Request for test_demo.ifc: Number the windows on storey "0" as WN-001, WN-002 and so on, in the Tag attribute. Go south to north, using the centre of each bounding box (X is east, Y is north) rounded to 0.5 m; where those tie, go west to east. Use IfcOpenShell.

First a look at what the model holds.

```python
import ifcopenshell
import ifcopenshell.util.element
import ifcopenshell.util.placement

model = ifcopenshell.open("test_demo.ifc")
print(model.schema)
storey = next(s for s in model.by_type("IfcBuildingStorey") if s.Name == "0")
windows = [e for e in ifcopenshell.util.element.get_decomposition(storey) if e.is_a("IfcWindow")]
for e in sorted(windows, key=lambda e: e.id()):
    origin = ifcopenshell.util.placement.get_local_placement(e.ObjectPlacement)[:3, 3]
    print(e.id(), e.Tag, e.Name, origin.round(2) + 0.0, sep=" | ")
```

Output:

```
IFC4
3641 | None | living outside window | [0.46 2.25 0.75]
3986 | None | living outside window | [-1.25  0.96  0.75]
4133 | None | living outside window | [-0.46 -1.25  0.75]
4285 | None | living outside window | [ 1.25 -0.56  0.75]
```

```python
import ifcopenshell
import ifcopenshell.geom
import ifcopenshell.util.element
import ifcopenshell.util.shape

model = ifcopenshell.open("test_demo.ifc")
settings = ifcopenshell.geom.settings()
settings.set("use-world-coords", True)


def centre(element):
    shape = ifcopenshell.geom.create_shape(settings, element)
    return ifcopenshell.util.shape.get_bbox_centroid(shape.geometry)


storey = next(s for s in model.by_type("IfcBuildingStorey") if s.Name == "0")
windows = [e for e in ifcopenshell.util.element.get_decomposition(storey) if e.is_a("IfcWindow")]

# Insertion points can sit at a corner or the storey origin, so sort by the geometry (in metres).
centres = {e: centre(e) for e in windows}
windows.sort(key=lambda e: (round(centres[e][1] / 0.5), centres[e][0]))

for i, e in enumerate(windows, start=1):
    number = f"WN-0{i:02d}"
    e.Tag = number
    print(e.id(), number)

model.write("test_demo_v2.ifc")
```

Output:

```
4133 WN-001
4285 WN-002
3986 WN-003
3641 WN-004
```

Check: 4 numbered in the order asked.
